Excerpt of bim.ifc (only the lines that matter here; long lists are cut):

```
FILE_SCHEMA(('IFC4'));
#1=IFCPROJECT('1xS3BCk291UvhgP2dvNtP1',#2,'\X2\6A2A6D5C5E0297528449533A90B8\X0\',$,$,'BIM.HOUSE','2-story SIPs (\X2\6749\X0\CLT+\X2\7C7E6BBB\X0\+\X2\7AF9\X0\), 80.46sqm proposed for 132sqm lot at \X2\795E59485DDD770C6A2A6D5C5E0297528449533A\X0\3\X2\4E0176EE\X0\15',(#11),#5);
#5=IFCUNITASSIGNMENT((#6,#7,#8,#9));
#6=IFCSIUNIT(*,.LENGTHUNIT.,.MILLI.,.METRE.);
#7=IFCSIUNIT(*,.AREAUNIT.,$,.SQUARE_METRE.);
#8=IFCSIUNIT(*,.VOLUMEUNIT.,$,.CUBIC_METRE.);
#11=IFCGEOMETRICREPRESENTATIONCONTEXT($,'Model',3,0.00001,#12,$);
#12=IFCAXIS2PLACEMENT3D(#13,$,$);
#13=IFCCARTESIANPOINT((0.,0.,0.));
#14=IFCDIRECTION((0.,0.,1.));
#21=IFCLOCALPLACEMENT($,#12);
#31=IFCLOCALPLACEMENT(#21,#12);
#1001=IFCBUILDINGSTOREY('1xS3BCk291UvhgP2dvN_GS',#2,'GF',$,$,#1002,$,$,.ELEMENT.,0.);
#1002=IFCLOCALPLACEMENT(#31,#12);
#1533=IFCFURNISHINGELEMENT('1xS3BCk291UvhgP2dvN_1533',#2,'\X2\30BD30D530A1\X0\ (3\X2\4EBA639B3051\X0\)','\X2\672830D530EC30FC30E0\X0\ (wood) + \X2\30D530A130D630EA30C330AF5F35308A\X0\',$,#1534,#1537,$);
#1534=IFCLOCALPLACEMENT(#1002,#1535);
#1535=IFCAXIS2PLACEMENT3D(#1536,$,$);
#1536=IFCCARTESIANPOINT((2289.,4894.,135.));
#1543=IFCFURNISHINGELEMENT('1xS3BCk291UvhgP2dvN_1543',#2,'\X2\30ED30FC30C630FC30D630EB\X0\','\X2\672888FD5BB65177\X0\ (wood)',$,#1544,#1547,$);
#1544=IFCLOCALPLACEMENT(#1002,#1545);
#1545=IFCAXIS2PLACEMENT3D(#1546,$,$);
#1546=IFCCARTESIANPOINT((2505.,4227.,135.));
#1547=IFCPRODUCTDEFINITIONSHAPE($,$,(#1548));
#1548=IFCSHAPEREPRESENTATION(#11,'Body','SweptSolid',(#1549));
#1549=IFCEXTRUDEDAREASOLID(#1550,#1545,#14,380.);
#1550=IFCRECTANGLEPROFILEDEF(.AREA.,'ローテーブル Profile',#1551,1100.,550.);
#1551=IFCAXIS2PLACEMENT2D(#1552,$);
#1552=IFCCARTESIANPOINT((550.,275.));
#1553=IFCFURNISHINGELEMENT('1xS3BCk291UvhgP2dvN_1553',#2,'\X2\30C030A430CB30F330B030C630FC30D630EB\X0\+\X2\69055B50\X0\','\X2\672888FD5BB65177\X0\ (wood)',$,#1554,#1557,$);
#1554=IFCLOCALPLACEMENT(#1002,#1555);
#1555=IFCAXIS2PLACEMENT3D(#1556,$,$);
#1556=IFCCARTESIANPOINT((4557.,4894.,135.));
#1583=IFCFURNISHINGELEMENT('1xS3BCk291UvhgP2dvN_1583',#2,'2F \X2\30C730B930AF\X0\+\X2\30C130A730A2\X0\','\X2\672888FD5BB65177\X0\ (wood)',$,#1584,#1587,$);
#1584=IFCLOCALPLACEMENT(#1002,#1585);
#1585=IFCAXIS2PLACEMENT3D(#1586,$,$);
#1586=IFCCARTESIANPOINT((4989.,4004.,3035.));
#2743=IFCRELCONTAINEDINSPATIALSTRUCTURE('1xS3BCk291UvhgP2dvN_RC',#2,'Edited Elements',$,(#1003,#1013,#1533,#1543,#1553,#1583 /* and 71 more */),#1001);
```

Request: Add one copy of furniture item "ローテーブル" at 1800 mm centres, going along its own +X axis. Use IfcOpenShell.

```python
import ifcopenshell
import ifcopenshell.api.geometry
import ifcopenshell.api.root
import ifcopenshell.util.element
import ifcopenshell.util.placement
import ifcopenshell.util.unit

model = ifcopenshell.open("bim.ifc")
unit_scale = ifcopenshell.util.unit.calculate_unit_scale(model)


def reuse_history(source, copy):
    """copy_class also copies each property set's owner history, people and application; keep the originals."""
    for rel in copy.IsDefinedBy:
        if rel.is_a("IfcRelDefinesByProperties") and (history := rel.RelatingPropertyDefinition.OwnerHistory):
            rel.RelatingPropertyDefinition.OwnerHistory = source.OwnerHistory
            ifcopenshell.util.element.remove_deep2(model, history)


source = model.by_guid("1xS3BCk291UvhgP2dvN_1543")
base = ifcopenshell.util.placement.get_local_placement(source.ObjectPlacement)
step = base[:3, 0] * 1.8 / unit_scale

for i in range(1, 2):
    copy = ifcopenshell.api.root.copy_class(model, product=source)
    copy.Representation = ifcopenshell.util.element.copy_deep(
        model, source.Representation, exclude=["IfcGeometricRepresentationContext", "IfcRepresentationMap"]
    )
    reuse_history(source, copy)
    matrix = base.copy()
    matrix[:3, 3] += i * step
    print("added at", matrix[:3, 3].round(3) + 0.0)
    ifcopenshell.api.geometry.edit_object_placement(model, product=copy, matrix=matrix, is_si=False)

model.write("bim_edited.ifc")
```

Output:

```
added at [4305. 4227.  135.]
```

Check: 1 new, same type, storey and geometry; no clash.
